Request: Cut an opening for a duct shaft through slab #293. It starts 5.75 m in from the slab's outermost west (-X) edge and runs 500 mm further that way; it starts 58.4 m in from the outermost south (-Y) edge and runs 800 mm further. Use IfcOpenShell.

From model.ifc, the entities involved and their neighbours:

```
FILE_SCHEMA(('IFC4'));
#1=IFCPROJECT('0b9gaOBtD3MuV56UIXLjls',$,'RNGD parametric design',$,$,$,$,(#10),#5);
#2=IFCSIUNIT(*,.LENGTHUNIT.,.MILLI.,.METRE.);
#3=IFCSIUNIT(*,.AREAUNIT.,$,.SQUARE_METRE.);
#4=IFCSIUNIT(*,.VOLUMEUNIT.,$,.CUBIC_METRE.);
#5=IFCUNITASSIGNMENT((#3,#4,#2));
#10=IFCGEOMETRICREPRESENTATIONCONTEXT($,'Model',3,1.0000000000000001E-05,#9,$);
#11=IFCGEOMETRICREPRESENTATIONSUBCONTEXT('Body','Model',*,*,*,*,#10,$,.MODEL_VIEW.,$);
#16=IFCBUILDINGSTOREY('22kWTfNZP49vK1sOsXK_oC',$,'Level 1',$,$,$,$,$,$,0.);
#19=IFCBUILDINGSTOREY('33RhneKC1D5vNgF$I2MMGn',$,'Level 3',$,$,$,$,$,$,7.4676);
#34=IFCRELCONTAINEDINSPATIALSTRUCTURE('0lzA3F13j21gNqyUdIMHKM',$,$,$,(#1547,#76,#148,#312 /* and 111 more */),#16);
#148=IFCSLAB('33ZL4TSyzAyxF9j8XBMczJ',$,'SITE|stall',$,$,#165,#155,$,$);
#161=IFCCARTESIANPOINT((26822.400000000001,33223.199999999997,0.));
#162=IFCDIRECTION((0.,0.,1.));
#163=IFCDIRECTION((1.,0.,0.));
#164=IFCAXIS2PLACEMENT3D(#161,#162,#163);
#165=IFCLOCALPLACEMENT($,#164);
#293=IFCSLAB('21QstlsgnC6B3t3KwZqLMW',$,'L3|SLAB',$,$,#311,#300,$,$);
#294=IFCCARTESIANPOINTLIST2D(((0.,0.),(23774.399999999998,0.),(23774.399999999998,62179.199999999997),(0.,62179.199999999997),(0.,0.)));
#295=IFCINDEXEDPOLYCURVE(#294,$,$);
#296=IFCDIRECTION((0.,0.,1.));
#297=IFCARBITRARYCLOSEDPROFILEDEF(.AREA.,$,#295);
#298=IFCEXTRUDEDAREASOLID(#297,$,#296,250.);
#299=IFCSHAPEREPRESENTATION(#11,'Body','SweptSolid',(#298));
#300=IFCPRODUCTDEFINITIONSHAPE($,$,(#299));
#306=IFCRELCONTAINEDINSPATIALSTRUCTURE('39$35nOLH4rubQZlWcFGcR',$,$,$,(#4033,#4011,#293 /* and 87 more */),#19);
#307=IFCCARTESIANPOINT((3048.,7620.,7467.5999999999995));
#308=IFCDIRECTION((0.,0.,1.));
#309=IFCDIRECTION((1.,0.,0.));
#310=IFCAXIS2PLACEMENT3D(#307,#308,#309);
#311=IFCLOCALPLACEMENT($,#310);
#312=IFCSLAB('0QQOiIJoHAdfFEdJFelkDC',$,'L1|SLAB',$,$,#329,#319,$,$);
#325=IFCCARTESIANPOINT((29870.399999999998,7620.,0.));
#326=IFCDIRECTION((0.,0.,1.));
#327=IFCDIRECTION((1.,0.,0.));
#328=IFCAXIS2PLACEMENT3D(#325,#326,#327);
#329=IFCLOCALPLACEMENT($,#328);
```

```python
import numpy as np
import ifcopenshell
import ifcopenshell.api.feature
import ifcopenshell.api.geometry
import ifcopenshell.api.root
import ifcopenshell.geom
import ifcopenshell.util.placement
import ifcopenshell.util.representation
import ifcopenshell.util.shape
import ifcopenshell.util.unit

model = ifcopenshell.open("model.ifc")
unit_scale = ifcopenshell.util.unit.calculate_unit_scale(model)
settings = ifcopenshell.geom.settings()


def volume(element):
    """Net volume in cubic metres, openings subtracted."""
    shape = ifcopenshell.geom.create_shape(settings, element)
    return ifcopenshell.util.shape.get_volume(shape.geometry)


slab = model.by_id(293)
before = volume(slab)

# Extent in the slab's own axes, in metres. The edges named are its -X and -Y sides.
slab_shape = ifcopenshell.geom.create_shape(settings, slab)
vertices = ifcopenshell.util.shape.get_vertices(slab_shape.geometry)
x_min, y_min, bottom = vertices.min(axis=0)
top = vertices[:, 2].max()

opening = ifcopenshell.api.root.create_entity(model, ifc_class="IfcOpeningElement", name="Duct shaft opening", predefined_type="OPENING")
context = ifcopenshell.util.representation.get_context(model, "Model", "Body", "MODEL_VIEW")
width, depth = 0.5, 0.8
outline = [(0.0, 0.0), (width, 0.0), (width, depth), (0.0, depth), (0.0, 0.0)]
# Overshoot both faces by 50 mm so the cut is clean.
shape = ifcopenshell.api.geometry.add_slab_representation(
    model, context=context, depth=top - bottom + 0.1, polyline=outline
)
ifcopenshell.api.geometry.assign_representation(model, product=opening, representation=shape)

matrix = ifcopenshell.util.placement.get_local_placement(slab.ObjectPlacement)
matrix[:, 3] = matrix @ np.append(np.array([x_min + 5.75, y_min + 58.4, bottom - 0.05]) / unit_scale, 1.0)
ifcopenshell.api.geometry.edit_object_placement(model, product=opening, matrix=matrix, is_si=False)
ifcopenshell.api.feature.add_feature(model, feature=opening, element=slab)

after = volume(slab)

print(f"slab volume {before:.3f} -> {after:.3f} m3")

model.write("model_updated.ifc")
```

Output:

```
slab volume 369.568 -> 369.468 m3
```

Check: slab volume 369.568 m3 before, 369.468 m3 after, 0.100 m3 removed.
